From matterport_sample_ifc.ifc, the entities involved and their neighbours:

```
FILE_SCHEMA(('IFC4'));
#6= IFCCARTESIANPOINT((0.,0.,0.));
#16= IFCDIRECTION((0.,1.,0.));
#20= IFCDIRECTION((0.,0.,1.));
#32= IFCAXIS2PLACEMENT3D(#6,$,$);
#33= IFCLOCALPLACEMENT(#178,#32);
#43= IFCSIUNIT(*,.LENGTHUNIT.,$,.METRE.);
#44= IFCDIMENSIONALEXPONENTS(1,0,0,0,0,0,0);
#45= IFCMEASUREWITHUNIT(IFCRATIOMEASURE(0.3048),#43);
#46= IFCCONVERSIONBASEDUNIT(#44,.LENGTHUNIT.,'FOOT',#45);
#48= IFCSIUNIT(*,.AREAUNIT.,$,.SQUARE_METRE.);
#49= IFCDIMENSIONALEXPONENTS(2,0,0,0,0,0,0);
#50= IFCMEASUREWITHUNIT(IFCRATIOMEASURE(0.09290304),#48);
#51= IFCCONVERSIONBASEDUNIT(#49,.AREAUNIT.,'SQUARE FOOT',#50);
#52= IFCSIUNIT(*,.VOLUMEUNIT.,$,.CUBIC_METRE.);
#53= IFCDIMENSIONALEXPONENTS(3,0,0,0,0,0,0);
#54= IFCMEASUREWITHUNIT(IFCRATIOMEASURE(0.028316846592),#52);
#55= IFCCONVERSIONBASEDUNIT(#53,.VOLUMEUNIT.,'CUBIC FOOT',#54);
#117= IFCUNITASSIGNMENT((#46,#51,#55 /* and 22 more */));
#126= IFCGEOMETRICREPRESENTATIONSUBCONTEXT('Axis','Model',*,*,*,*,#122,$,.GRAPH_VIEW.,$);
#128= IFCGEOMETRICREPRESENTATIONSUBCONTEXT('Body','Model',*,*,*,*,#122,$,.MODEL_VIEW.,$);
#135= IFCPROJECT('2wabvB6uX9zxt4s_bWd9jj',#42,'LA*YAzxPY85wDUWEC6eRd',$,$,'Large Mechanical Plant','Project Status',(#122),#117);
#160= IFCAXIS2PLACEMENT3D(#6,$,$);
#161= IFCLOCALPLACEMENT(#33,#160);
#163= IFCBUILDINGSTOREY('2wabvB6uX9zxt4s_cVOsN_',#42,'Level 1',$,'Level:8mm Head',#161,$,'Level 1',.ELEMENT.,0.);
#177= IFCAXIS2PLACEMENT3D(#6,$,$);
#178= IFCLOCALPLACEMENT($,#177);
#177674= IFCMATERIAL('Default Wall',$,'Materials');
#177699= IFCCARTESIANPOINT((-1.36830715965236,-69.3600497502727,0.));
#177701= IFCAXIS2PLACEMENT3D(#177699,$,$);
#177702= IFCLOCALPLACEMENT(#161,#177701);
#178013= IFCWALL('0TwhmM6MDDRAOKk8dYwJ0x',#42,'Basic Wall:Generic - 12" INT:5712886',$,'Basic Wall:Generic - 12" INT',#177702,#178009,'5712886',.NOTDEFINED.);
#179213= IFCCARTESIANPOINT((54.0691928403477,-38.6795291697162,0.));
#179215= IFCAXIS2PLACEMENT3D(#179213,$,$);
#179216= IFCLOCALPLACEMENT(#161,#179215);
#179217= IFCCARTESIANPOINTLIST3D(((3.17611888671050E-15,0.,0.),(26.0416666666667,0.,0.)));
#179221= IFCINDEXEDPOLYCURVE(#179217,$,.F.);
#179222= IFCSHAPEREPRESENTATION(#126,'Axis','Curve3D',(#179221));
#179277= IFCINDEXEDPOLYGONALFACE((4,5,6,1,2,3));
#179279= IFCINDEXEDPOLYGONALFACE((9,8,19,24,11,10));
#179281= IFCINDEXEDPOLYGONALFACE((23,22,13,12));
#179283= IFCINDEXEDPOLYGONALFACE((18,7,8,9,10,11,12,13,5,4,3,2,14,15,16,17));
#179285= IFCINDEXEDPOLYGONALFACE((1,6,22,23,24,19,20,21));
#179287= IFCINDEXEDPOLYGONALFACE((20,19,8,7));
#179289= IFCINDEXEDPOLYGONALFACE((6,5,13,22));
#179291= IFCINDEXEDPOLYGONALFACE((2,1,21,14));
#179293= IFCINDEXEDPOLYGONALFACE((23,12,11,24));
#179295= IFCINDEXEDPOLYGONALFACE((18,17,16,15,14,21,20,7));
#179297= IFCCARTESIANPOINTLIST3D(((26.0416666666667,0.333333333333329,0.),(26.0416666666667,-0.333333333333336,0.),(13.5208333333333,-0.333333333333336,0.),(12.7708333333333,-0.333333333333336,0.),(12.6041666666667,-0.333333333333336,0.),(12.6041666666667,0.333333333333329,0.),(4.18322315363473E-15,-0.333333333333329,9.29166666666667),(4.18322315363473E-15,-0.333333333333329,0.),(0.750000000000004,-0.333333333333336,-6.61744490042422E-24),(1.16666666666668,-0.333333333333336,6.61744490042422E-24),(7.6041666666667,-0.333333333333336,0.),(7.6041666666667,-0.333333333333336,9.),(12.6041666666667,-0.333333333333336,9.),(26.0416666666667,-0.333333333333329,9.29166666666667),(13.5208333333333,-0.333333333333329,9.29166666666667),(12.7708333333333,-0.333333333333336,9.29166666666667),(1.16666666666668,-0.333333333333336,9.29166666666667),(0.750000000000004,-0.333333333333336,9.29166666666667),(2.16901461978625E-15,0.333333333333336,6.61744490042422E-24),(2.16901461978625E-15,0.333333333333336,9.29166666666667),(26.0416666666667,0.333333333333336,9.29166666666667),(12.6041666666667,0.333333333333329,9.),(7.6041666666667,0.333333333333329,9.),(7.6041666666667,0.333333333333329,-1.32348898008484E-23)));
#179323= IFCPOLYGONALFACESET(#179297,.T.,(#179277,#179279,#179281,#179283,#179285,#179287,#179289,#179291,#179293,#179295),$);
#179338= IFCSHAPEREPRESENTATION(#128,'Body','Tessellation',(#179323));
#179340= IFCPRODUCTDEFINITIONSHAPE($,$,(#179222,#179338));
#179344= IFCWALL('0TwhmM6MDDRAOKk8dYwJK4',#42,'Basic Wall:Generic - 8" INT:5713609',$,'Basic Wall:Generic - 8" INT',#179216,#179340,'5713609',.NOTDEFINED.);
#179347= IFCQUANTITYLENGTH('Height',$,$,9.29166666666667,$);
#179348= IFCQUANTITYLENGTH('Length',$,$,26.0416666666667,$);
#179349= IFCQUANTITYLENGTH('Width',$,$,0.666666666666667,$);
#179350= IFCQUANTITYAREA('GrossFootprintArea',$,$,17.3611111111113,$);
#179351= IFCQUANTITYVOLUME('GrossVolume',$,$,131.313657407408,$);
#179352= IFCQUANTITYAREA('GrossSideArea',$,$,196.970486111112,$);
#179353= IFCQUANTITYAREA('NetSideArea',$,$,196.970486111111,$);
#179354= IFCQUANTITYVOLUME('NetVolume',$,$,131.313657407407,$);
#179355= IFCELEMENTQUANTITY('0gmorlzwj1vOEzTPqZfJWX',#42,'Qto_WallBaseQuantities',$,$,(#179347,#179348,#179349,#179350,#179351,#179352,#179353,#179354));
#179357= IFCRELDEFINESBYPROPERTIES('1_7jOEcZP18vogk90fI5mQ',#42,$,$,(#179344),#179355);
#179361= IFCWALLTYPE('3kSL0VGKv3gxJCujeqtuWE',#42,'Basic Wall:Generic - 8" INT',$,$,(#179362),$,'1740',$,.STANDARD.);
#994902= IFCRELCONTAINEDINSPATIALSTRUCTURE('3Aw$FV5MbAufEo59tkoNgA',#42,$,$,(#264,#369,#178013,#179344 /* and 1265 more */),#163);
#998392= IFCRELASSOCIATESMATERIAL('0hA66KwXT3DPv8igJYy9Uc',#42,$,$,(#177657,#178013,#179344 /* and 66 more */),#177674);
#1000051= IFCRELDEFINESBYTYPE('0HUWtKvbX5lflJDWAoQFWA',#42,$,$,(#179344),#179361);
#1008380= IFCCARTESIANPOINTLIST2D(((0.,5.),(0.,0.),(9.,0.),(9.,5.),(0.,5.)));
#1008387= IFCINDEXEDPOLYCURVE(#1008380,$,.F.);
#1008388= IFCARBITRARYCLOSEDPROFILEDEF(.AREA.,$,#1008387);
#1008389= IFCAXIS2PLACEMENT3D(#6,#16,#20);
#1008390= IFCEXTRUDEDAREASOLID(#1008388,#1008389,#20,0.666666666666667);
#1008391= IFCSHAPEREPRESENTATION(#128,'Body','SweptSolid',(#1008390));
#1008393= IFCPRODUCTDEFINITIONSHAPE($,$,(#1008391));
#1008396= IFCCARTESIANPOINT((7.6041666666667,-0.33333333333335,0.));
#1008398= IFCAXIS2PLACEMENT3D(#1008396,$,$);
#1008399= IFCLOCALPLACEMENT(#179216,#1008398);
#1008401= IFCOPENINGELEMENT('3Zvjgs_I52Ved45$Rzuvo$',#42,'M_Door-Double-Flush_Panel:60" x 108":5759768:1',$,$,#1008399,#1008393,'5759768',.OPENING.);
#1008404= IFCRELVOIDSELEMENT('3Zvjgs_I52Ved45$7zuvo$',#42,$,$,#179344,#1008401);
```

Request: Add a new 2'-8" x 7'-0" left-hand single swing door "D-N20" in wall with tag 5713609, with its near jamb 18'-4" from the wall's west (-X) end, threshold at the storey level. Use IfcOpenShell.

```python
import numpy as np
import ifcopenshell
import ifcopenshell.api.feature
import ifcopenshell.api.geometry
import ifcopenshell.api.pset
import ifcopenshell.api.root
import ifcopenshell.api.spatial
import ifcopenshell.geom
import ifcopenshell.util.element
import ifcopenshell.util.placement
import ifcopenshell.util.representation
import ifcopenshell.util.shape
import ifcopenshell.util.unit

model = ifcopenshell.open("matterport_sample_ifc.ifc")
unit_scale = ifcopenshell.util.unit.calculate_unit_scale(model)
area_scale = ifcopenshell.util.unit.calculate_unit_scale(model, "AREAUNIT")
volume_scale = ifcopenshell.util.unit.calculate_unit_scale(model, "VOLUMEUNIT")
settings = ifcopenshell.geom.settings()


def volume(element):
    """Net volume in cubic metres, openings subtracted."""
    shape = ifcopenshell.geom.create_shape(settings, element)
    return ifcopenshell.util.shape.get_volume(shape.geometry)


wall = model.by_id(179344)
storey = ifcopenshell.util.element.get_container(wall, ifc_class="IfcBuildingStorey")
context = ifcopenshell.util.representation.get_context(model, "Model", "Body", "MODEL_VIEW")
before = volume(wall)

width, height, from_end, sill = 0.8128, 2.1336, 5.588, 0.0  # metres

# The wall runs along its own X axis, and the end named is its -X end.
wall_shape = ifcopenshell.geom.create_shape(settings, wall)
x, y, z = ifcopenshell.util.shape.get_vertices(wall_shape.geometry).T
start = x.min() + from_end
face, thickness = float(y.min()), float(y.max() - y.min())
wall_matrix = ifcopenshell.util.placement.get_local_placement(wall.ObjectPlacement)
level = ifcopenshell.util.placement.get_local_placement(storey.ObjectPlacement)[2, 3]


def in_wall(x, y):
    """Placement at x, y metres in the wall's axes, at sill height."""
    matrix = wall_matrix.copy()
    matrix[:, 3] = wall_matrix @ np.array([x / unit_scale, y / unit_scale, 0.0, 1.0])
    matrix[2, 3] = level + sill / unit_scale
    return matrix


# Opening: a box that overshoots both wall faces by 50 mm.
opening = ifcopenshell.api.root.create_entity(model, ifc_class="IfcOpeningElement", predefined_type="OPENING")
box = ifcopenshell.api.geometry.add_wall_representation(
    model, context=context, length=width, height=height, thickness=thickness + 0.1
)
ifcopenshell.api.geometry.assign_representation(model, product=opening, representation=box)
ifcopenshell.api.geometry.edit_object_placement(model, product=opening, matrix=in_wall(start, face - 0.05), is_si=False)
ifcopenshell.api.feature.add_feature(model, feature=opening, element=wall)

door = ifcopenshell.api.root.create_entity(model, ifc_class="IfcDoor", name="D-N20", predefined_type="DOOR")
door.OverallWidth, door.OverallHeight = width / unit_scale, height / unit_scale
door.OperationType = "SINGLE_SWING_LEFT"
body = ifcopenshell.api.geometry.add_door_representation(
    model,
    context=context,
    overall_width=door.OverallWidth,
    overall_height=door.OverallHeight,
    operation_type="SINGLE_SWING_LEFT",
    lining_properties={"LiningDepth": thickness / unit_scale, "ThresholdDepth": thickness / unit_scale},
)
ifcopenshell.api.geometry.assign_representation(model, product=door, representation=body)
ifcopenshell.api.spatial.assign_container(model, products=[door], relating_structure=storey)
ifcopenshell.api.feature.add_filling(model, opening=opening, element=door)

# The lining spans the wall, so the door starts at the wall face.
ifcopenshell.api.geometry.edit_object_placement(model, product=door, matrix=in_wall(start, face), is_si=False)

after = volume(wall)

# Update the wall's stored quantities.
qto = model.by_id(ifcopenshell.util.element.get_pset(wall, "Qto_WallBaseQuantities", should_inherit=False)["id"])
ifcopenshell.api.pset.edit_qto(model, qto=qto, properties={
    "NetSideArea": after / thickness / area_scale,
    "NetVolume": after / volume_scale,
})

print(f"wall volume {before:.3f} -> {after:.3f} m3")

model.write("matterport_sample_ifc_v2.ifc")
```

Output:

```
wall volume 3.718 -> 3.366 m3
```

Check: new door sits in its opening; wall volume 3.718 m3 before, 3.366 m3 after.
